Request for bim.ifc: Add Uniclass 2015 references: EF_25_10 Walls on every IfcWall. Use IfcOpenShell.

First a look at what the model holds.

```python
import ifcopenshell

model = ifcopenshell.open("bim.ifc")
print(model.schema)
print("classifications:", [c.Name for c in model.by_type("IfcClassification")])
for ifc_class in ("IfcDoor", "IfcRoof", "IfcStair", "IfcWall", "IfcWindow"):
    print(ifc_class, len(model.by_type(ifc_class)))
```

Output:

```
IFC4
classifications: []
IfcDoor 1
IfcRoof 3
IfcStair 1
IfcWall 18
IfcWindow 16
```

```python
import ifcopenshell
import ifcopenshell.api.classification

model = ifcopenshell.open("bim.ifc")

system = ifcopenshell.api.classification.add_classification(model, classification="Uniclass 2015")

codes = {
    "IfcWall": ("EF_25_10", "Walls"),
}
for ifc_class, (code, name) in codes.items():
    products = model.by_type(ifc_class)
    ifcopenshell.api.classification.add_reference(
        model, products=products, classification=system, identification=code, name=name
    )
    print(code, len(products))

model.write("bim_updated.ifc")
```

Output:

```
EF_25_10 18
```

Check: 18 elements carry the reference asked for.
